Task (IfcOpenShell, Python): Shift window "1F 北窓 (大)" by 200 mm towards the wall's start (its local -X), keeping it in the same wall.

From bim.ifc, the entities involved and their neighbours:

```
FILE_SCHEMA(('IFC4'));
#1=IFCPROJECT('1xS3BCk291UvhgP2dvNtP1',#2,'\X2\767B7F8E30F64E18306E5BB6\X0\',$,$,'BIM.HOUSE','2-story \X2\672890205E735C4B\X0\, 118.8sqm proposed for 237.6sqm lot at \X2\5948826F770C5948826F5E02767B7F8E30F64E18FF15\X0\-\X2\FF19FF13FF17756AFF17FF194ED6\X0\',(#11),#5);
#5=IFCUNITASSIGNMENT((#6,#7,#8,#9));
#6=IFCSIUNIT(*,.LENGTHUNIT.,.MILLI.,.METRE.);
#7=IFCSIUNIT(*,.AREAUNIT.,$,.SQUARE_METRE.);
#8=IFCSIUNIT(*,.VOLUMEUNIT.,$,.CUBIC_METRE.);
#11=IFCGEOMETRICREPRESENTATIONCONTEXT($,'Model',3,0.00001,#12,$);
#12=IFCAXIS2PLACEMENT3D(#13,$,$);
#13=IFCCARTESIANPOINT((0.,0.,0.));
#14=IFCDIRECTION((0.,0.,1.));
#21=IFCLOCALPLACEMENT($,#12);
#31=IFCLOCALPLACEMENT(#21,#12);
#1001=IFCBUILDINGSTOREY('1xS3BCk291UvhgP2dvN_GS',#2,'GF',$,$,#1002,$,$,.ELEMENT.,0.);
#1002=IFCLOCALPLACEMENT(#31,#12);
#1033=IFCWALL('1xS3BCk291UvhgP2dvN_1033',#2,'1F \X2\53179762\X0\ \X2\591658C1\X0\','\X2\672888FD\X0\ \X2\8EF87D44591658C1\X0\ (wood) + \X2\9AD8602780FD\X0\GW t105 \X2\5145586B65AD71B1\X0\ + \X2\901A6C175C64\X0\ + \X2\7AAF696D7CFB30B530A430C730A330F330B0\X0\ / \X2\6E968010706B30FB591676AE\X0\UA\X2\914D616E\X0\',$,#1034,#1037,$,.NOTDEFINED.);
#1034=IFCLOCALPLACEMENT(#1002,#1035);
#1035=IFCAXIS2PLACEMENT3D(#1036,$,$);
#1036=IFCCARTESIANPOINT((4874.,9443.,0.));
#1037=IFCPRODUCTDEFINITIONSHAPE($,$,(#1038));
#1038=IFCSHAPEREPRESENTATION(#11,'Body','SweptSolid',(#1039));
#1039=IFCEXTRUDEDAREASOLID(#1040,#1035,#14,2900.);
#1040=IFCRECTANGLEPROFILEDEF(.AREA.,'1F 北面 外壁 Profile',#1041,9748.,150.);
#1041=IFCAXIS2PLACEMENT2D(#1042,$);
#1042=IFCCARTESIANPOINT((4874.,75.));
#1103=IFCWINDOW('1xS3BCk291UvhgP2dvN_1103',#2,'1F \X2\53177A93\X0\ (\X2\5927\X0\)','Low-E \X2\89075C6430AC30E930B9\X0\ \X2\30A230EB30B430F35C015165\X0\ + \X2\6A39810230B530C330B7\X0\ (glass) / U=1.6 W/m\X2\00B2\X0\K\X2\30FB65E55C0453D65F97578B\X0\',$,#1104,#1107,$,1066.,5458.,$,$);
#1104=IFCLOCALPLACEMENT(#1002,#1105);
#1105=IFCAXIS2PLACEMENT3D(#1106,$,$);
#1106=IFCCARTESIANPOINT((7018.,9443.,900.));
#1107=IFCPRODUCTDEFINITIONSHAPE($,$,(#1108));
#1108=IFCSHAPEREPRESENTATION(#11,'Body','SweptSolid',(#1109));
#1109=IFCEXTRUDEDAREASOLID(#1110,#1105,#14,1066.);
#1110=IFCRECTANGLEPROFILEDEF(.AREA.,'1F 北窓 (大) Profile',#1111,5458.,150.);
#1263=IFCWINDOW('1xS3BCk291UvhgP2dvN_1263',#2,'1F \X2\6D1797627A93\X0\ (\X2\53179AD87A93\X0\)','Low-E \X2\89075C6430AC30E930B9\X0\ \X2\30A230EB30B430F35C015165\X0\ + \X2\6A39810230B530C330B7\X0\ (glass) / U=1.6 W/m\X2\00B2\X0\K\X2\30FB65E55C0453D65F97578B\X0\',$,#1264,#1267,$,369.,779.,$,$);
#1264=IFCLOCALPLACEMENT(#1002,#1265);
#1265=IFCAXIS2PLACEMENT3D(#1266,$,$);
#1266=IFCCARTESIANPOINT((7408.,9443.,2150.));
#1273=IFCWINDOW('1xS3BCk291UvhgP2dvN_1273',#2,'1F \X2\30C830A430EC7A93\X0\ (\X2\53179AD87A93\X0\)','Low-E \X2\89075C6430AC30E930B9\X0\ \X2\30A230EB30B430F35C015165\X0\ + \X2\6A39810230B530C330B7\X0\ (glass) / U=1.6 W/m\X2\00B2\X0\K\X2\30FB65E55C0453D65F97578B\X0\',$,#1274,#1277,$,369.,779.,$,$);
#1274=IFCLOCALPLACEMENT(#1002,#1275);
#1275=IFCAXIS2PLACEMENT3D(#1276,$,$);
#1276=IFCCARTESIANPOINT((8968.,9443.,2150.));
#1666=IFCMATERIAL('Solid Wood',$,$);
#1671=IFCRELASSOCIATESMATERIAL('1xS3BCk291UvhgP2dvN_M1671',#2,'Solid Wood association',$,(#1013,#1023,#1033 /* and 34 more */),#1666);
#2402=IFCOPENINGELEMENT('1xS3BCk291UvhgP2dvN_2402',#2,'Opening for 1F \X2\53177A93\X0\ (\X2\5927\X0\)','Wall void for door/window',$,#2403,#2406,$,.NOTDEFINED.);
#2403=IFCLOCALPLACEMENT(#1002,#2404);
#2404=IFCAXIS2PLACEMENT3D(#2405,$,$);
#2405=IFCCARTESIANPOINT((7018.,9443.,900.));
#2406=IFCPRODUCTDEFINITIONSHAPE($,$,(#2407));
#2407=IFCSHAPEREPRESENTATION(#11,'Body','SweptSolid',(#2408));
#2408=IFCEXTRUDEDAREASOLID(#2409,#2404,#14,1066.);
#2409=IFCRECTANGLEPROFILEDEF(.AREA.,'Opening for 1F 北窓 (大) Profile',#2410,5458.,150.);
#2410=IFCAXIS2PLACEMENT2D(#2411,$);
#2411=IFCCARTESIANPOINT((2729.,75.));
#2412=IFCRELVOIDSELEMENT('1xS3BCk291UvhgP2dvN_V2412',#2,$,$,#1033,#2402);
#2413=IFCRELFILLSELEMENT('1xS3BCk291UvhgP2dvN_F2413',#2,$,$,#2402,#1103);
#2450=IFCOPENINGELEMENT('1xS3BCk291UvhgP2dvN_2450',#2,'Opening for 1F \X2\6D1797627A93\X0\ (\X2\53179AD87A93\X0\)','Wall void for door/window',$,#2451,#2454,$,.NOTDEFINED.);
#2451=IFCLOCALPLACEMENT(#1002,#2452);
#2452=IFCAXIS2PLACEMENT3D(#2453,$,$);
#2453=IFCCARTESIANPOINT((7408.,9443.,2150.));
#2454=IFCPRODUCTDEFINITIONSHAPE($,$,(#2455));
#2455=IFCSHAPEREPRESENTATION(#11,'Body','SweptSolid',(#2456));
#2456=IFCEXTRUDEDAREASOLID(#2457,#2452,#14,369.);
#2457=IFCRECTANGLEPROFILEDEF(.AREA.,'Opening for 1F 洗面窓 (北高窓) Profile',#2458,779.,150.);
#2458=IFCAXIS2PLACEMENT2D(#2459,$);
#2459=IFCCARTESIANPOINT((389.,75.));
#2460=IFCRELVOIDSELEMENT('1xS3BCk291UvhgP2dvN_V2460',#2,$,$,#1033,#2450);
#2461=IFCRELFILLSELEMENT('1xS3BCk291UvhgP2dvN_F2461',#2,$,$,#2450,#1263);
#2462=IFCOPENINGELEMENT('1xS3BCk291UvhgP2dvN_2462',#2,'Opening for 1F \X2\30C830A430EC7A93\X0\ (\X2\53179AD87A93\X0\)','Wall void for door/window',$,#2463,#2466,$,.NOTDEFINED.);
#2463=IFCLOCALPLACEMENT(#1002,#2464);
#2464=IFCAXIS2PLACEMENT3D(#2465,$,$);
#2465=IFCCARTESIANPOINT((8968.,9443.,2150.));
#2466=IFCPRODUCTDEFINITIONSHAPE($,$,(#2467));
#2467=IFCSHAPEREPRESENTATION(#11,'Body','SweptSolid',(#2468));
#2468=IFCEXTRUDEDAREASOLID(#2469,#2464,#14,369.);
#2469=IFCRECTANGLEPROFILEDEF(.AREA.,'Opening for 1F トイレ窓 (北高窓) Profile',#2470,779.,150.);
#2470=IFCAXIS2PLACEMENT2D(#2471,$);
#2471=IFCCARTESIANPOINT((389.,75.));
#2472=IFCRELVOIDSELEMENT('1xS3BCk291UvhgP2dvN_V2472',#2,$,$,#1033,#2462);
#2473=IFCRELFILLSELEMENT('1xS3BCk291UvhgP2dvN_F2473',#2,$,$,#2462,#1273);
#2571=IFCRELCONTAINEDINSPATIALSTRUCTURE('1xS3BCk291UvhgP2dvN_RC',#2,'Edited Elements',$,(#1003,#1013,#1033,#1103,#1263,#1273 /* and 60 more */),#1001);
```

```python
import ifcopenshell
import ifcopenshell.api.geometry
import ifcopenshell.util.placement
import ifcopenshell.util.unit

model = ifcopenshell.open("bim.ifc")
unit_scale = ifcopenshell.util.unit.calculate_unit_scale(model)

window = model.by_guid("1xS3BCk291UvhgP2dvN_1103")
opening = window.FillsVoids[0].RelatingOpeningElement
wall = opening.VoidsElements[0].RelatingBuildingElement

wall_matrix = ifcopenshell.util.placement.get_local_placement(wall.ObjectPlacement)
shift = wall_matrix[:3, 0] * -0.2 / unit_scale
before = ifcopenshell.util.placement.get_local_placement(window.ObjectPlacement)[:3, 3].copy()

# The window is not placed relative to its opening, so move both.
for product in (opening, window):
    matrix = ifcopenshell.util.placement.get_local_placement(product.ObjectPlacement)
    matrix[:3, 3] += shift
    ifcopenshell.api.geometry.edit_object_placement(model, product=product, matrix=matrix, is_si=False)

after = ifcopenshell.util.placement.get_local_placement(window.ObjectPlacement)[:3, 3]
print("window moved by", (after - before).round(3) + 0.0)

model.write("bim_rev.ifc")
```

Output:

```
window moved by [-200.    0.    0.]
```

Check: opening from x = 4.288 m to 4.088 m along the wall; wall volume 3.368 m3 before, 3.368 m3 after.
